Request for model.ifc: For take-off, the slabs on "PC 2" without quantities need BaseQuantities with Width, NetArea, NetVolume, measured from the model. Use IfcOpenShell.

First a look at what the model holds.

```python
import ifcopenshell
import ifcopenshell.util.element
import ifcopenshell.util.unit

model = ifcopenshell.open("model.ifc")
print(model.schema)
for unit_type in ("LENGTHUNIT", "AREAUNIT", "VOLUMEUNIT"):
    print(unit_type, ifcopenshell.util.unit.calculate_unit_scale(model, unit_type))
storey = next(s for s in model.by_type("IfcBuildingStorey") if s.Name == "PC 2")
slabs = [e for e in ifcopenshell.util.element.get_decomposition(storey) if e.is_a("IfcSlab")]
for e in sorted(slabs, key=lambda e: e.id()):
    print(e.id(), e.is_a(), e.Name, list(ifcopenshell.util.element.get_psets(e, qtos_only=True)), sep=" | ")
```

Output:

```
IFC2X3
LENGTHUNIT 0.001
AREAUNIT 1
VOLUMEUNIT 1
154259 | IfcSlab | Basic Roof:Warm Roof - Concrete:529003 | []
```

```python
import ifcopenshell
import ifcopenshell.api.pset
import ifcopenshell.geom
import ifcopenshell.util.element
import ifcopenshell.util.shape
import ifcopenshell.util.unit

model = ifcopenshell.open("model.ifc")
unit_scale = ifcopenshell.util.unit.calculate_unit_scale(model)
area_scale = ifcopenshell.util.unit.calculate_unit_scale(model, "AREAUNIT")
volume_scale = ifcopenshell.util.unit.calculate_unit_scale(model, "VOLUMEUNIT")
settings = ifcopenshell.geom.settings()

storey = next(s for s in model.by_type("IfcBuildingStorey") if s.Name == "PC 2")
slabs = [e for e in ifcopenshell.util.element.get_decomposition(storey) if e.is_a("IfcSlab")]

for e in sorted(slabs, key=lambda e: e.id()):
    if ifcopenshell.util.element.get_psets(e, qtos_only=True, should_inherit=False):
        continue
    # Geometry comes back in metres, in the element's own axes.
    shape = ifcopenshell.geom.create_shape(settings, e)
    values = {
        "Width": ifcopenshell.util.shape.get_z(shape.geometry) / unit_scale,
        "NetArea": ifcopenshell.util.shape.get_footprint_area(shape.geometry) / area_scale,
        "NetVolume": ifcopenshell.util.shape.get_volume(shape.geometry) / volume_scale,
    }
    qto = ifcopenshell.api.pset.add_qto(model, product=e, name="BaseQuantities")
    ifcopenshell.api.pset.edit_qto(model, qto=qto, properties=values)
    print(e.id(), {k: round(v, 3) for k, v in values.items()})

model.write("model_rev.ifc")
```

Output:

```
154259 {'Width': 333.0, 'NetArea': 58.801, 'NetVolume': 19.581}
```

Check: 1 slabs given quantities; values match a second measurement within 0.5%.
